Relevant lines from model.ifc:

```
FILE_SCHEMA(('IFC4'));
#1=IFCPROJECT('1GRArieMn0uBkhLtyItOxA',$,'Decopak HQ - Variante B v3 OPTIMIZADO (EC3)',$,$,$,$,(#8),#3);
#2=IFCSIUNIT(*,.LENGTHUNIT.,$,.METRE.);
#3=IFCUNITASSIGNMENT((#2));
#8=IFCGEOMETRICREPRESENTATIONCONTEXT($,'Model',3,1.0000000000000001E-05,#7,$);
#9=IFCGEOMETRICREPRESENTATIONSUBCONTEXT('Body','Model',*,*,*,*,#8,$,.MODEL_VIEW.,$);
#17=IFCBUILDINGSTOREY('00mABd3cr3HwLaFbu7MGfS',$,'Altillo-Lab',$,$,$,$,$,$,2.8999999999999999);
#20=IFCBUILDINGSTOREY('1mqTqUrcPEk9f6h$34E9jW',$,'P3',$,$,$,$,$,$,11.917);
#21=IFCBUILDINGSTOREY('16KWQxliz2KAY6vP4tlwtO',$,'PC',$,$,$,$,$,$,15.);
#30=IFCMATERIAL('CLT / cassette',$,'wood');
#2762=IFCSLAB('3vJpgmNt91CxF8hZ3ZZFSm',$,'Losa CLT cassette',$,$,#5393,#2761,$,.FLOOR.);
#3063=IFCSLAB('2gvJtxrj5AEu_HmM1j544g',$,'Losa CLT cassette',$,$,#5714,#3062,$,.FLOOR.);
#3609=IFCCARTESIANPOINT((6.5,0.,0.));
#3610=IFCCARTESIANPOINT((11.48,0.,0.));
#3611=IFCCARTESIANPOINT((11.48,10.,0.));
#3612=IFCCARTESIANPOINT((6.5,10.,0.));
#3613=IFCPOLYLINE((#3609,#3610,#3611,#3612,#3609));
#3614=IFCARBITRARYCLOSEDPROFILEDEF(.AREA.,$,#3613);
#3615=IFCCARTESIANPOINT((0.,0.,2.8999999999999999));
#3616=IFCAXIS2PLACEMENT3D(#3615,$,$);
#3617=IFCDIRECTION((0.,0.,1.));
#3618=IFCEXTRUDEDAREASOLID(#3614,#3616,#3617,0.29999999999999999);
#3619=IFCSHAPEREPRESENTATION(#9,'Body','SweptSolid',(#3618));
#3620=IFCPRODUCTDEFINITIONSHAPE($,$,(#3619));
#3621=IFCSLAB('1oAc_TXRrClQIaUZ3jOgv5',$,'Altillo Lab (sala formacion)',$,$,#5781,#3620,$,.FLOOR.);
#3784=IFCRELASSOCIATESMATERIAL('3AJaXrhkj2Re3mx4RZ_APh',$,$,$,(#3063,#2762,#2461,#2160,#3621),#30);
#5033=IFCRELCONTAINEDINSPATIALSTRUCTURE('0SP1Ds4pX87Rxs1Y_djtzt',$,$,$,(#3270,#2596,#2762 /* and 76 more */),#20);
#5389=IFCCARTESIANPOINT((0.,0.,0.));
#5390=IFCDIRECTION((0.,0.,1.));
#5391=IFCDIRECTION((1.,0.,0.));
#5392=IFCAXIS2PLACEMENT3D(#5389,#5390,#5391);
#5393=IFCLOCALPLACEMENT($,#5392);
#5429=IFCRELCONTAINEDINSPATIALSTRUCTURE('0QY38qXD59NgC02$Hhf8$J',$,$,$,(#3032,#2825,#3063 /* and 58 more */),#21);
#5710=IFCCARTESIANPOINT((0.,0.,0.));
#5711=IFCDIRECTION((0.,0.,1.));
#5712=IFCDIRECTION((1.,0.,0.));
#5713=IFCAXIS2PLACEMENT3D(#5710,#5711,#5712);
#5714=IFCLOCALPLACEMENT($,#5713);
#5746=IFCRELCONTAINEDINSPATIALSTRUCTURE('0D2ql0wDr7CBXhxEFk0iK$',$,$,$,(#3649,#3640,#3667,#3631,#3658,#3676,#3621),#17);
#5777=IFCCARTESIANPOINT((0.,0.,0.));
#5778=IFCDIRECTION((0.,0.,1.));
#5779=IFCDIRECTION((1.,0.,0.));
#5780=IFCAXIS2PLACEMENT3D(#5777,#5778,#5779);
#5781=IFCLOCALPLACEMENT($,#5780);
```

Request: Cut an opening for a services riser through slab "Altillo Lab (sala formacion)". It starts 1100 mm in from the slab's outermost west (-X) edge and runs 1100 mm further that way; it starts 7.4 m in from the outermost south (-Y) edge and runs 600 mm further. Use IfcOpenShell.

```python
import numpy as np
import ifcopenshell
import ifcopenshell.api.feature
import ifcopenshell.api.geometry
import ifcopenshell.api.root
import ifcopenshell.geom
import ifcopenshell.util.placement
import ifcopenshell.util.representation
import ifcopenshell.util.shape
import ifcopenshell.util.unit

model = ifcopenshell.open("model.ifc")
unit_scale = ifcopenshell.util.unit.calculate_unit_scale(model)
settings = ifcopenshell.geom.settings()


def volume(element):
    """Net volume in cubic metres, openings subtracted."""
    shape = ifcopenshell.geom.create_shape(settings, element)
    return ifcopenshell.util.shape.get_volume(shape.geometry)


slab = model.by_guid("1oAc_TXRrClQIaUZ3jOgv5")
before = volume(slab)

# Extent in the slab's own axes, in metres. The edges named are its -X and -Y sides.
slab_shape = ifcopenshell.geom.create_shape(settings, slab)
vertices = ifcopenshell.util.shape.get_vertices(slab_shape.geometry)
x_min, y_min, bottom = vertices.min(axis=0)
top = vertices[:, 2].max()

opening = ifcopenshell.api.root.create_entity(model, ifc_class="IfcOpeningElement", name="Services riser opening", predefined_type="OPENING")
context = ifcopenshell.util.representation.get_context(model, "Model", "Body", "MODEL_VIEW")
width, depth = 1.1, 0.6
outline = [(0.0, 0.0), (width, 0.0), (width, depth), (0.0, depth), (0.0, 0.0)]
# Overshoot both faces by 50 mm so the cut is clean.
shape = ifcopenshell.api.geometry.add_slab_representation(
    model, context=context, depth=top - bottom + 0.1, polyline=outline
)
ifcopenshell.api.geometry.assign_representation(model, product=opening, representation=shape)

matrix = ifcopenshell.util.placement.get_local_placement(slab.ObjectPlacement)
matrix[:, 3] = matrix @ np.append(np.array([x_min + 1.1, y_min + 7.4, bottom - 0.05]) / unit_scale, 1.0)
ifcopenshell.api.geometry.edit_object_placement(model, product=opening, matrix=matrix, is_si=False)
ifcopenshell.api.feature.add_feature(model, feature=opening, element=slab)

after = volume(slab)

print(f"slab volume {before:.3f} -> {after:.3f} m3")

model.write("model_edited.ifc")
```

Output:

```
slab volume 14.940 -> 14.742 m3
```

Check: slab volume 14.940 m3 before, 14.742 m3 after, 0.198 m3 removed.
